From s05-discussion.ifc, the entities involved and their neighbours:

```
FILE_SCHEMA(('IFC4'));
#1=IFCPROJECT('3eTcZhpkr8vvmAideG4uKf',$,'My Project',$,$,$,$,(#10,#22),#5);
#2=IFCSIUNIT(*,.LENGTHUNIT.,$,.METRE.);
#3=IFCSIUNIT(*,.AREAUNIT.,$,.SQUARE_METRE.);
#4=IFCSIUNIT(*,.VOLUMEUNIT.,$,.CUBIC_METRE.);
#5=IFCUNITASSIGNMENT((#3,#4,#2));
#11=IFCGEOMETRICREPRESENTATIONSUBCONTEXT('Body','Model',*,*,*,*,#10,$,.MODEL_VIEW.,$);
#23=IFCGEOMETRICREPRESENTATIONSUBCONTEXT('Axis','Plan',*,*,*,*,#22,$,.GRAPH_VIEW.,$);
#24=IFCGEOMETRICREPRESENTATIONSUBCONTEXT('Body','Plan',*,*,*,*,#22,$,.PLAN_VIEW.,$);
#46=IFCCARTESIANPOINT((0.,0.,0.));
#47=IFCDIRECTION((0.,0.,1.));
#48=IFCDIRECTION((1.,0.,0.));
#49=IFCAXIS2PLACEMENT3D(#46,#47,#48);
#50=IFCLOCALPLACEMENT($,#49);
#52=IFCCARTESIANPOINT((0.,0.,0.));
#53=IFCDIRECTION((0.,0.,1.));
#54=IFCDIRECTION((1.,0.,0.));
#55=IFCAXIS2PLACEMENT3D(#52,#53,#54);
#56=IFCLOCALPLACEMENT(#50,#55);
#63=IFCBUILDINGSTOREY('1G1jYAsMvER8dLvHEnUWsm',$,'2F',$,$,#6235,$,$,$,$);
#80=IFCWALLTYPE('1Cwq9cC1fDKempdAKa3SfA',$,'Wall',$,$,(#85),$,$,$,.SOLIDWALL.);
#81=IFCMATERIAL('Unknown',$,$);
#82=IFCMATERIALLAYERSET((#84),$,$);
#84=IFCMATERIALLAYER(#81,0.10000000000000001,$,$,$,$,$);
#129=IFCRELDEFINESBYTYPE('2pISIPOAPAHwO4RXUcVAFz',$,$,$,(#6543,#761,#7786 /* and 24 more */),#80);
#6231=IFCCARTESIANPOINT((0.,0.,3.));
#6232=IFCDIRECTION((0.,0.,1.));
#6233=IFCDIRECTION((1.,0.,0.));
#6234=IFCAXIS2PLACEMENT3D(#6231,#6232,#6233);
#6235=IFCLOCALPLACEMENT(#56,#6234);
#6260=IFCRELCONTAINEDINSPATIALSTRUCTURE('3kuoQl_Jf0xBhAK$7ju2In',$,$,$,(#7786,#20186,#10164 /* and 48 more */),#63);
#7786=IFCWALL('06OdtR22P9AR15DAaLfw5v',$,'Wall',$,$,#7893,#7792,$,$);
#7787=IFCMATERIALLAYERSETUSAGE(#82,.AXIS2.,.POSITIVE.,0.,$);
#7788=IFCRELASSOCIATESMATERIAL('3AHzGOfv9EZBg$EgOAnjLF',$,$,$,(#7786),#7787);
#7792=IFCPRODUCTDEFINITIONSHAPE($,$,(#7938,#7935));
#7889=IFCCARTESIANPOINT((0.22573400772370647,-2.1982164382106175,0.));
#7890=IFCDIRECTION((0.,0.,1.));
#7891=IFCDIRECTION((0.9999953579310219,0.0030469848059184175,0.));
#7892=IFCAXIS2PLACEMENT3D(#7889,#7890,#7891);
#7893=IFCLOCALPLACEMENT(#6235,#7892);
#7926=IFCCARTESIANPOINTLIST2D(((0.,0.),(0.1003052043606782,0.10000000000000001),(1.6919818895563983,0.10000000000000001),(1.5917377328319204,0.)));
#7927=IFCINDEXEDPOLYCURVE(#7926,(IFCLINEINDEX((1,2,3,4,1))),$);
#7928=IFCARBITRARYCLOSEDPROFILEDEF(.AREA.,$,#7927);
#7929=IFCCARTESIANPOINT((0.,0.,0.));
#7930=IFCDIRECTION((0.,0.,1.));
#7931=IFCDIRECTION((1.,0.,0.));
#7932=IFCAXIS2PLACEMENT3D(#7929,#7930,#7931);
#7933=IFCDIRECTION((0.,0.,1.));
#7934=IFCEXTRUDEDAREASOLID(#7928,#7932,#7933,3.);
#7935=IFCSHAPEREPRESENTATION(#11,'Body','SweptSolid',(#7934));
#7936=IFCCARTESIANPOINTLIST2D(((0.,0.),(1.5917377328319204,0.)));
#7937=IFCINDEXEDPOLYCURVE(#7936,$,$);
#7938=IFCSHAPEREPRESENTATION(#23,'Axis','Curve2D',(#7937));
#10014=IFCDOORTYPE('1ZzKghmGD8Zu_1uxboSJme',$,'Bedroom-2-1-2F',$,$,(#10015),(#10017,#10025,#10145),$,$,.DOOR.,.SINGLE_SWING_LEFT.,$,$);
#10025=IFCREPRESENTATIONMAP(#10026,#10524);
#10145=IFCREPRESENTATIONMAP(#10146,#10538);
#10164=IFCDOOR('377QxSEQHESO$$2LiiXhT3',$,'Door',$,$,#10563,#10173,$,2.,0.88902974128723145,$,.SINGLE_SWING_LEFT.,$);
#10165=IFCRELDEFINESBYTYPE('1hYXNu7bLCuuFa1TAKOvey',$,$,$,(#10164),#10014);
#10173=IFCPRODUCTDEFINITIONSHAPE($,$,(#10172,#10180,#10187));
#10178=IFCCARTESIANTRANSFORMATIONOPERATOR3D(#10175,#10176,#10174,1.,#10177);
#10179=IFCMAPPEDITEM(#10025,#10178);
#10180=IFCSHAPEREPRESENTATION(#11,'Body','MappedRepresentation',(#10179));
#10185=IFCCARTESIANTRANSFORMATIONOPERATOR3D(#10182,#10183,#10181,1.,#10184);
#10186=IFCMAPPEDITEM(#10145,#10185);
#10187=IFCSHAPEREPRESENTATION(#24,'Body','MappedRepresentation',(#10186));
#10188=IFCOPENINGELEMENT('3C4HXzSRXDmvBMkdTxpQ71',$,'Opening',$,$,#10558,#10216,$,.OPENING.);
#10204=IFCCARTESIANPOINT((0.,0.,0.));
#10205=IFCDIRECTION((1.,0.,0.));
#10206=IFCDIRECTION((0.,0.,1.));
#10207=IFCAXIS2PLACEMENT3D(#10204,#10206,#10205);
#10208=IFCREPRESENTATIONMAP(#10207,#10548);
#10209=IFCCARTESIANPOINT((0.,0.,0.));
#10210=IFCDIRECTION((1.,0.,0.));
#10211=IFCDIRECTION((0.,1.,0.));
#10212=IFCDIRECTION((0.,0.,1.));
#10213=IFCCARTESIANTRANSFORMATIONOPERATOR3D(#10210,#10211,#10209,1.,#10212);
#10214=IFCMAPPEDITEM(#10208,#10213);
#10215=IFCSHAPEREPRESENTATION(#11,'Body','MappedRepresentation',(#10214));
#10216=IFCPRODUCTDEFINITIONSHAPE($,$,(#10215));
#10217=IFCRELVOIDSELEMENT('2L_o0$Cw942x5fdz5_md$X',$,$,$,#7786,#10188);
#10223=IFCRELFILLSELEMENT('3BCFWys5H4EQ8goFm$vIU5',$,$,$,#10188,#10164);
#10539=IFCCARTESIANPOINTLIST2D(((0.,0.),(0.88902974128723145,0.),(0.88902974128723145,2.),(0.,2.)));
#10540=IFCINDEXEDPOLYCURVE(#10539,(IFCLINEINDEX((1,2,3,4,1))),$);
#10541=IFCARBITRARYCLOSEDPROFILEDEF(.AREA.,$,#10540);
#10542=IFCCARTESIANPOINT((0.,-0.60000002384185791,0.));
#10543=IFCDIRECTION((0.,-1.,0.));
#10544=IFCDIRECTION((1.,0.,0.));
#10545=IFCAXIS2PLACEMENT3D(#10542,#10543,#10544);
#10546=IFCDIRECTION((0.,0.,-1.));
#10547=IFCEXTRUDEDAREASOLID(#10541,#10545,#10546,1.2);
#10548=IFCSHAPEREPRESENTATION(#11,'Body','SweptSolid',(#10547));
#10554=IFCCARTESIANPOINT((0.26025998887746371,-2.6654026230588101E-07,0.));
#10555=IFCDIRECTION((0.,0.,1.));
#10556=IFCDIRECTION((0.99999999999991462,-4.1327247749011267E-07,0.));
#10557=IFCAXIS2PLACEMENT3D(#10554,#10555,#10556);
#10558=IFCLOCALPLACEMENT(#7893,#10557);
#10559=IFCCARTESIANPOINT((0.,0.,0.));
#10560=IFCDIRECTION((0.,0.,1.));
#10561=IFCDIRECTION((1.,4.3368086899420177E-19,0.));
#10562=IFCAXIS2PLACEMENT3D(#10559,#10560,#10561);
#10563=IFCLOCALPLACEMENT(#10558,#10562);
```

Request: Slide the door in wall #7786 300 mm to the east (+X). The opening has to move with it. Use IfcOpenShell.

```python
import ifcopenshell
import ifcopenshell.api.geometry
import ifcopenshell.util.placement

model = ifcopenshell.open("s05-discussion.ifc")

door = model.by_guid("377QxSEQHESO$$2LiiXhT3")
opening = door.FillsVoids[0].RelatingOpeningElement
wall = opening.VoidsElements[0].RelatingBuildingElement

wall_matrix = ifcopenshell.util.placement.get_local_placement(wall.ObjectPlacement)
shift = wall_matrix[:3, 0] * 0.3
before = ifcopenshell.util.placement.get_local_placement(door.ObjectPlacement)[:3, 3].copy()

# The door is placed relative to its opening, so it follows when the opening moves.
matrix = ifcopenshell.util.placement.get_local_placement(opening.ObjectPlacement)
matrix[:3, 3] += shift
ifcopenshell.api.geometry.edit_object_placement(
    model, product=opening, matrix=matrix, is_si=False, should_transform_children=True
)

after = ifcopenshell.util.placement.get_local_placement(door.ObjectPlacement)[:3, 3]
print("door moved by", (after - before).round(3) + 0.0)

model.write("s05-discussion_updated.ifc")
```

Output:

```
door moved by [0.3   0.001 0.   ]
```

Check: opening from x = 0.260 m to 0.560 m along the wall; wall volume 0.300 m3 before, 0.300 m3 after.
